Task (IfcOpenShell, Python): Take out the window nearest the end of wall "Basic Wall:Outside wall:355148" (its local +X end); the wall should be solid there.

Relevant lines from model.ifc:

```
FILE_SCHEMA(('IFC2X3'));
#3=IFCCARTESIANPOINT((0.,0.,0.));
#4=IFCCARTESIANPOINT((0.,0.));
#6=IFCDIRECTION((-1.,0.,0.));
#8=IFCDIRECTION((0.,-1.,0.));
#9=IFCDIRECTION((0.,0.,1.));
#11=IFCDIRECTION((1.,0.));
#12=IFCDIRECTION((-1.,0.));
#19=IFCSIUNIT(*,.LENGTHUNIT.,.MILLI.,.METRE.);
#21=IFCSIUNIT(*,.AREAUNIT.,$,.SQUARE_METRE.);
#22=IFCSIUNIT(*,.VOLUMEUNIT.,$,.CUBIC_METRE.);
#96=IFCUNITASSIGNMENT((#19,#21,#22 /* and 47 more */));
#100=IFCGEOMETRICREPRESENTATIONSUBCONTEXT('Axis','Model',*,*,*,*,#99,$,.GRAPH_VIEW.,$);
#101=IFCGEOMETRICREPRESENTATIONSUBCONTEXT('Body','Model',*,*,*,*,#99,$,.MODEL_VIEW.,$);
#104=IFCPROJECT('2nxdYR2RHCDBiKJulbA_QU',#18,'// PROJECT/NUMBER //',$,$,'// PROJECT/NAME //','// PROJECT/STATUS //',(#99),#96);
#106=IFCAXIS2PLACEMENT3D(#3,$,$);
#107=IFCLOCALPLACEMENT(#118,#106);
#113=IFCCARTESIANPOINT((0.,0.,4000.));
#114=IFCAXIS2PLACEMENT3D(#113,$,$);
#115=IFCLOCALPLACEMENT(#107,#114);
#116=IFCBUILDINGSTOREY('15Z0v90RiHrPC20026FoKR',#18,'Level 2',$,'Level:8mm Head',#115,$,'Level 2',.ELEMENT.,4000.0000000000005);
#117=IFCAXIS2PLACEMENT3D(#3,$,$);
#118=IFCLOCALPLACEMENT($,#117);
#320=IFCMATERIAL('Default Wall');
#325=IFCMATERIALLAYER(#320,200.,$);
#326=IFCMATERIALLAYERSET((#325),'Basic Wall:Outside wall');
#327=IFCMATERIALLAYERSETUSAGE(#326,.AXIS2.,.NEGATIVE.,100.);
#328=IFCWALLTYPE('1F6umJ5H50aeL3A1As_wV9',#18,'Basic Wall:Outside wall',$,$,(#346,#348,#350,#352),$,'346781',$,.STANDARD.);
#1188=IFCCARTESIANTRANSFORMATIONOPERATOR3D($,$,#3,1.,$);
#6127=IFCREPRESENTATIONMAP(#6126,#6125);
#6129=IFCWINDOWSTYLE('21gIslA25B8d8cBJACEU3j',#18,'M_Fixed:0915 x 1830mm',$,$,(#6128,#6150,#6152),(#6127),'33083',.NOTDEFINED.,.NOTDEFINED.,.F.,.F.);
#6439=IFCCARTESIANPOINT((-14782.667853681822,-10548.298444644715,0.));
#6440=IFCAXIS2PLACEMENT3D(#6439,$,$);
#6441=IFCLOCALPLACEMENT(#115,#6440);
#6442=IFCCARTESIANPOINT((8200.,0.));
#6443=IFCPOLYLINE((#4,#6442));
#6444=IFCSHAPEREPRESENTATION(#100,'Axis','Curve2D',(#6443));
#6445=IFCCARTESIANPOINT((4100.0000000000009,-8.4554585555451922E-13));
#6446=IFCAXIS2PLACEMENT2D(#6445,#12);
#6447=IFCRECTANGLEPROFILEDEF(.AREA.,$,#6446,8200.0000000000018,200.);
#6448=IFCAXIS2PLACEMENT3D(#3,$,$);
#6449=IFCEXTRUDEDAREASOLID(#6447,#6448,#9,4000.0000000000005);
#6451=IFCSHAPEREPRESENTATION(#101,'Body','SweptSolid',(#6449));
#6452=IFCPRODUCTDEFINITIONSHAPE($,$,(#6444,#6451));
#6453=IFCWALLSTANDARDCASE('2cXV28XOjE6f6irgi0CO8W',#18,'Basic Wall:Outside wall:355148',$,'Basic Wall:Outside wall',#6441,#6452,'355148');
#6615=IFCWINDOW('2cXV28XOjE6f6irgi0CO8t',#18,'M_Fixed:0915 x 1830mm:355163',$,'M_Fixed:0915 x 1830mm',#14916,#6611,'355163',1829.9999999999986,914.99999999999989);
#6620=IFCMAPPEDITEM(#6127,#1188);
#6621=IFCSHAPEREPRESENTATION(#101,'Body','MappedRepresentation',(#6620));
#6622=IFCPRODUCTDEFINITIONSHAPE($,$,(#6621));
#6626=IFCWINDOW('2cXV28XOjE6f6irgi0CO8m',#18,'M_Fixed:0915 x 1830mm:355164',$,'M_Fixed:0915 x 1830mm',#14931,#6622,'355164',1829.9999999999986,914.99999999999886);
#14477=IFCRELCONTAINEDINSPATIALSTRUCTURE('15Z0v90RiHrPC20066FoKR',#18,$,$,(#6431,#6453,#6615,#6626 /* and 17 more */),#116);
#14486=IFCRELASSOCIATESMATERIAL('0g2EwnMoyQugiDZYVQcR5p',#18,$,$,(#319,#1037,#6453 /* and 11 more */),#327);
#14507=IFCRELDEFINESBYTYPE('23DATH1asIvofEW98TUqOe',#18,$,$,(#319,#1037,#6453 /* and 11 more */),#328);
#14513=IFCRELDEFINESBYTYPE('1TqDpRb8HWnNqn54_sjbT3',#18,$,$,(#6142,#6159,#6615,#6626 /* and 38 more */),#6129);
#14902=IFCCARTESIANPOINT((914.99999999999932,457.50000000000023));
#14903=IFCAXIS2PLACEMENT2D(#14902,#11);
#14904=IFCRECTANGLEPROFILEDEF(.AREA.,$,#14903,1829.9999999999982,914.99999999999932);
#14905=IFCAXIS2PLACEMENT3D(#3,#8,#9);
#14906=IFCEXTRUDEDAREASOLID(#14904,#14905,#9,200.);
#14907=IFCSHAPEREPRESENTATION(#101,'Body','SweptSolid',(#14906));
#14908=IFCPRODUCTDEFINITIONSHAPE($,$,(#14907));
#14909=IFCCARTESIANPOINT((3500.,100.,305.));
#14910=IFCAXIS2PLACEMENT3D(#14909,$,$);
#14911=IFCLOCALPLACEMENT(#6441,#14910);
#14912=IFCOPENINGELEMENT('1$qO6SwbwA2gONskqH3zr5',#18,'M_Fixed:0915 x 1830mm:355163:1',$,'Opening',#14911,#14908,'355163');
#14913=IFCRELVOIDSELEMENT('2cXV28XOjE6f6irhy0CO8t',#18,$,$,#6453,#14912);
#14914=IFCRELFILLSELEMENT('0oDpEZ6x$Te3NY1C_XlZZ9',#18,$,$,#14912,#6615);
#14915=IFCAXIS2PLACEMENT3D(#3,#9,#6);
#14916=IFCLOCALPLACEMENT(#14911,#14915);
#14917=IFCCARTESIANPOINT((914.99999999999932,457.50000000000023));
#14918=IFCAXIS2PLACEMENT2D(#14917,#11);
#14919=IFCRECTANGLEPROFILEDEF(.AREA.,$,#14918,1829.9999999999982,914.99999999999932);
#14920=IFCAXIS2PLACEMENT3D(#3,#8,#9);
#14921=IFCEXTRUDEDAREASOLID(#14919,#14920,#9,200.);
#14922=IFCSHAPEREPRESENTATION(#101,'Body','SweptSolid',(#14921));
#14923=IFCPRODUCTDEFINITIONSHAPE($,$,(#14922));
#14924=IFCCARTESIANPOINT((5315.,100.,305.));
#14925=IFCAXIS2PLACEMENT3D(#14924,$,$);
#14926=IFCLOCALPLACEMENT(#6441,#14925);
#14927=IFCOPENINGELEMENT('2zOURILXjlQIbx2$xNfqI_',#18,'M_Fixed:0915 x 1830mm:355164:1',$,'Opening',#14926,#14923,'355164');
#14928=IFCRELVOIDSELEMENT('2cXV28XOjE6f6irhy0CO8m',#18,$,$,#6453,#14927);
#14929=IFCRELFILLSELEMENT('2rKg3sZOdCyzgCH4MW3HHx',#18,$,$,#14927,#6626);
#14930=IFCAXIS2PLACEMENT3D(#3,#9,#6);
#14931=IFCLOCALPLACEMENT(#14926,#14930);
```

```python
import ifcopenshell
import ifcopenshell.api.feature
import ifcopenshell.api.root
import ifcopenshell.geom
import ifcopenshell.util.shape

model = ifcopenshell.open("model.ifc")
settings = ifcopenshell.geom.settings()


def volume(element):
    """Net volume in cubic metres, openings subtracted."""
    shape = ifcopenshell.geom.create_shape(settings, element)
    return ifcopenshell.util.shape.get_volume(shape.geometry)


window = model.by_id(6626)
opening = window.FillsVoids[0].RelatingOpeningElement
wall = opening.VoidsElements[0].RelatingBuildingElement
before = volume(wall)

ifcopenshell.api.root.remove_product(model, product=window)
ifcopenshell.api.feature.remove_feature(model, feature=opening)

after = volume(wall)

print(f"wall volume {before:.3f} -> {after:.3f} m3")

model.write("model_v2.ifc")
```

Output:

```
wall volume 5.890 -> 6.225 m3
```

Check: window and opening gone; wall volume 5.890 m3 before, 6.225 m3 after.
